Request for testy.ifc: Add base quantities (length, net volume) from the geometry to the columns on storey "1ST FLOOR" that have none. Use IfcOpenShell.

First a look at what the model holds.

```python
import ifcopenshell
import ifcopenshell.util.element
import ifcopenshell.util.unit

model = ifcopenshell.open("testy.ifc")
print(model.schema)
for unit_type in ("LENGTHUNIT", "AREAUNIT", "VOLUMEUNIT"):
    print(unit_type, ifcopenshell.util.unit.calculate_unit_scale(model, unit_type))
storey = next(s for s in model.by_type("IfcBuildingStorey") if s.Name == "1ST FLOOR")
columns = [e for e in ifcopenshell.util.element.get_decomposition(storey) if e.is_a("IfcColumn")]
for e in sorted(columns, key=lambda e: e.id()):
    print(e.id(), e.is_a(), e.Name, list(ifcopenshell.util.element.get_psets(e, qtos_only=True)), sep=" | ")
```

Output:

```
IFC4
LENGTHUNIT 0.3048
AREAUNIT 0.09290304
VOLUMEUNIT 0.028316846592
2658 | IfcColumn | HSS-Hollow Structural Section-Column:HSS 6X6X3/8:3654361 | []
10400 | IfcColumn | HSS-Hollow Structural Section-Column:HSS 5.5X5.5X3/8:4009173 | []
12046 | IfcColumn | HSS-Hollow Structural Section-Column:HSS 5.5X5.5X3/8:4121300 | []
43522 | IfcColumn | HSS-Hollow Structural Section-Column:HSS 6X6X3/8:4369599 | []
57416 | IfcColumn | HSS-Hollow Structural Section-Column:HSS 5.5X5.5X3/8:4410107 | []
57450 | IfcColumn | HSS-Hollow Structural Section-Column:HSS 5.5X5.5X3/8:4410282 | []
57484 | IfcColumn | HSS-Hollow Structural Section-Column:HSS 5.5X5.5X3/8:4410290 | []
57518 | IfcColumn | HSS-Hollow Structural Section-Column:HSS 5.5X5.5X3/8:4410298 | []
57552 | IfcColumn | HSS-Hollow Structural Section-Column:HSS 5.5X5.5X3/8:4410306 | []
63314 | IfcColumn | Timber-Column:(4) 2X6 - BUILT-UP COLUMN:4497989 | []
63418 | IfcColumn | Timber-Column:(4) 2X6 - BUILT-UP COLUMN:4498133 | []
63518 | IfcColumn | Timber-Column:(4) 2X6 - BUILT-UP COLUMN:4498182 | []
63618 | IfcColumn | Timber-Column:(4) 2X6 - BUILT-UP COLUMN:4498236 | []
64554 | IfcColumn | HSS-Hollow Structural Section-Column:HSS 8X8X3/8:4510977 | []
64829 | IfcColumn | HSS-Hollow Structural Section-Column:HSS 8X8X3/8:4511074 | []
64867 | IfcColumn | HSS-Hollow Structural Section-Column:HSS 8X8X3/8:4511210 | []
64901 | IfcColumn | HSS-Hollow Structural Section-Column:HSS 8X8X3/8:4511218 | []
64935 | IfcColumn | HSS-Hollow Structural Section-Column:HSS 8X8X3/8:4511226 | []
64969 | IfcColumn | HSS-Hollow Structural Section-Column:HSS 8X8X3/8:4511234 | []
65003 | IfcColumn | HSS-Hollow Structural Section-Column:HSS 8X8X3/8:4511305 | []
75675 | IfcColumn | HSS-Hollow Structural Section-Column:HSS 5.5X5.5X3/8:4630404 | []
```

```python
import ifcopenshell
import ifcopenshell.api.pset
import ifcopenshell.geom
import ifcopenshell.util.element
import ifcopenshell.util.shape
import ifcopenshell.util.unit

model = ifcopenshell.open("testy.ifc")
unit_scale = ifcopenshell.util.unit.calculate_unit_scale(model)
volume_scale = ifcopenshell.util.unit.calculate_unit_scale(model, "VOLUMEUNIT")
settings = ifcopenshell.geom.settings()

storey = next(s for s in model.by_type("IfcBuildingStorey") if s.Name == "1ST FLOOR")
columns = [e for e in ifcopenshell.util.element.get_decomposition(storey) if e.is_a("IfcColumn")]

for e in sorted(columns, key=lambda e: e.id()):
    if ifcopenshell.util.element.get_psets(e, qtos_only=True, should_inherit=False):
        continue
    # Geometry comes back in metres, in the element's own axes.
    shape = ifcopenshell.geom.create_shape(settings, e)
    values = {
        "Length": ifcopenshell.util.shape.get_z(shape.geometry) / unit_scale,
        "NetVolume": ifcopenshell.util.shape.get_volume(shape.geometry) / volume_scale,
    }
    qto = ifcopenshell.api.pset.add_qto(model, product=e, name="Qto_ColumnBaseQuantities")
    ifcopenshell.api.pset.edit_qto(model, qto=qto, properties=values)
    print(e.id(), {k: round(v, 3) for k, v in values.items()})

model.write("testy_edited.ifc")
```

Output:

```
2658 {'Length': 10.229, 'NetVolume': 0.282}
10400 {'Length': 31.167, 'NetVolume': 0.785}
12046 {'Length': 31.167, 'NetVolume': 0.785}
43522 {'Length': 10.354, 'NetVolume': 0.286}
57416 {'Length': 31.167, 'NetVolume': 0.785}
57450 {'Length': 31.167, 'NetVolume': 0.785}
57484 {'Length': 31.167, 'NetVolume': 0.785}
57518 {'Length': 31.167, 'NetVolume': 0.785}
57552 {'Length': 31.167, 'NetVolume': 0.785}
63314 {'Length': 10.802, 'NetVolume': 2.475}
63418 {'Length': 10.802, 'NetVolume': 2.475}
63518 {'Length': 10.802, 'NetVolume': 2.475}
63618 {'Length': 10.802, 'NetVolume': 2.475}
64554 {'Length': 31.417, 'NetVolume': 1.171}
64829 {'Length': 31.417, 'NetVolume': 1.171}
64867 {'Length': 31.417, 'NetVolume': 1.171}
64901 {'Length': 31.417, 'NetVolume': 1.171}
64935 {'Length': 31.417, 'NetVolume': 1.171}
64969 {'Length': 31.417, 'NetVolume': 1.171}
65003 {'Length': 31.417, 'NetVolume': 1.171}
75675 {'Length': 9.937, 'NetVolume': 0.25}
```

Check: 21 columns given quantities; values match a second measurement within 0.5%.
